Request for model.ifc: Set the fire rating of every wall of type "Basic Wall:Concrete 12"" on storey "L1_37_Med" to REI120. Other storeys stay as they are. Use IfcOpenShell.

First a look at what the model holds.

```python
import ifcopenshell
import ifcopenshell.util.element

model = ifcopenshell.open("model.ifc")
print(model.schema)
storey = next(s for s in model.by_type("IfcBuildingStorey") if s.Name == "L1_37_Med")
walls = [e for e in ifcopenshell.util.element.get_decomposition(storey) if e.is_a("IfcWall")]
seen = {}
for e in walls:
    element_type = ifcopenshell.util.element.get_type(e)
    key = (element_type.Name if element_type != e and element_type else None, ifcopenshell.util.element.get_pset(e, "Pset_WallCommon", "FireRating"))
    seen[key] = seen.get(key, 0) + 1
for (name, value), count in sorted(seen.items(), key=str):
    print(count, "x", name, "|", value)
```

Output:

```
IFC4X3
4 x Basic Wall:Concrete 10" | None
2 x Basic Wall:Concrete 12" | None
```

```python
import ifcopenshell
import ifcopenshell.api.pset
import ifcopenshell.util.element

model = ifcopenshell.open("model.ifc")

storey = next(s for s in model.by_type("IfcBuildingStorey") if s.Name == "L1_37_Med")
walls = [e for e in ifcopenshell.util.element.get_decomposition(storey) if e.is_a("IfcWall")]

count = 0
for e in walls:
    element_type = ifcopenshell.util.element.get_type(e)
    if element_type in (None, e) or element_type.Name != 'Basic Wall:Concrete 12"':
        continue
    # add_pset returns the element's existing set when there is one.
    pset = ifcopenshell.api.pset.add_pset(model, product=e, name="Pset_WallCommon")
    ifcopenshell.api.pset.edit_pset(model, pset=pset, properties={"FireRating": "REI120"})
    count += 1

print(count, "walls updated")

model.write("model_updated.ifc")
```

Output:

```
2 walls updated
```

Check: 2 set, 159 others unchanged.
